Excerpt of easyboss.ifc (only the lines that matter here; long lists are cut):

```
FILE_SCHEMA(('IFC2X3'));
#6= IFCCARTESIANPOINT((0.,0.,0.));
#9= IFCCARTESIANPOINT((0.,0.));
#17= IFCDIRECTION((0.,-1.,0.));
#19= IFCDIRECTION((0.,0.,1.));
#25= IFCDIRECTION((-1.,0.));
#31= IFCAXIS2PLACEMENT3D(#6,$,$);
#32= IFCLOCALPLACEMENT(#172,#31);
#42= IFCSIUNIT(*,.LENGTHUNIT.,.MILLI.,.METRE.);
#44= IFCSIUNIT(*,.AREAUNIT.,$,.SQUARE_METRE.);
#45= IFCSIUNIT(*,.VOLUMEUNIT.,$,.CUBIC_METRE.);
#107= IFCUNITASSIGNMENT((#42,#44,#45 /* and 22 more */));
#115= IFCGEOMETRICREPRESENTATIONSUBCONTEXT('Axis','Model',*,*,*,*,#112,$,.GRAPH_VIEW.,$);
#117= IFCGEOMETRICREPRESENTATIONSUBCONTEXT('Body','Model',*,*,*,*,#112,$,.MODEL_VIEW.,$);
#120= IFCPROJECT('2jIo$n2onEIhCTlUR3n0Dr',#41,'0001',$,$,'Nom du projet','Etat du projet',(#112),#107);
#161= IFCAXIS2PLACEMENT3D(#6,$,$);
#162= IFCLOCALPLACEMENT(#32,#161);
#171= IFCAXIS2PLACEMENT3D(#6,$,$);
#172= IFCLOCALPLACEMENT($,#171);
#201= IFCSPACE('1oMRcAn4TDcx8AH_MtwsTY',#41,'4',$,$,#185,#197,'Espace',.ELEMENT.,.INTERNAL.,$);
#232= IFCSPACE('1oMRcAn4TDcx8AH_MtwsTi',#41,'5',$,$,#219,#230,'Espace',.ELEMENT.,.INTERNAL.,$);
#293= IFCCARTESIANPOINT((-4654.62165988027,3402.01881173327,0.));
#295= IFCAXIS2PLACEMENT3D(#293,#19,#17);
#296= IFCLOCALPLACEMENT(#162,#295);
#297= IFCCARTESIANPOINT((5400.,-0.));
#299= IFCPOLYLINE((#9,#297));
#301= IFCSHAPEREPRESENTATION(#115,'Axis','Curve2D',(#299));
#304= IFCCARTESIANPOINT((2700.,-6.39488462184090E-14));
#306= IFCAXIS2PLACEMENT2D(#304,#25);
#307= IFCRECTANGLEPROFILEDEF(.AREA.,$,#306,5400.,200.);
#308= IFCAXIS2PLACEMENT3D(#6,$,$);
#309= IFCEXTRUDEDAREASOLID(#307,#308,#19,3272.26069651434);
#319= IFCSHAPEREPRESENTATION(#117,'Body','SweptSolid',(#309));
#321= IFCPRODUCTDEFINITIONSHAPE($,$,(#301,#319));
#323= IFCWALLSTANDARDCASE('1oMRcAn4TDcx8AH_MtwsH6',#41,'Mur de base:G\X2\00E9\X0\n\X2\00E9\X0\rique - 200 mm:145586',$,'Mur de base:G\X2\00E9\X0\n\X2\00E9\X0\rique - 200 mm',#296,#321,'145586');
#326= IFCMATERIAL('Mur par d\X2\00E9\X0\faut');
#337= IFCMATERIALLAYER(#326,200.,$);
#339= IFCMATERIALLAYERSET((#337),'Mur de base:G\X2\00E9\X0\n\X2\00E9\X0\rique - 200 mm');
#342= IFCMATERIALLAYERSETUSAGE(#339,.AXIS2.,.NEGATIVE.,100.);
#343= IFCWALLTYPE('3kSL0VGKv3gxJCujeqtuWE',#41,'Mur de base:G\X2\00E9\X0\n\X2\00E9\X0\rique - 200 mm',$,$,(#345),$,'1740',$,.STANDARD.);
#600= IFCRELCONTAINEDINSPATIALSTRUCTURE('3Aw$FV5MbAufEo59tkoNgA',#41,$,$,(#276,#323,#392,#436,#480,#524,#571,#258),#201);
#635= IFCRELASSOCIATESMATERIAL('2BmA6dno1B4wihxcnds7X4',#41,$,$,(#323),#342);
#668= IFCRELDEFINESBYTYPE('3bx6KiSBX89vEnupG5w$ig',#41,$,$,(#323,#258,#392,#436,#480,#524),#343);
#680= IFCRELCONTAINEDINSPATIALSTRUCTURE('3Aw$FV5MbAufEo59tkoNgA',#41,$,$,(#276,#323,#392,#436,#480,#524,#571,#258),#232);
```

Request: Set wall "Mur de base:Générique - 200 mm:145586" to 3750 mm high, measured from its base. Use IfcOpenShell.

```python
import ifcopenshell
import ifcopenshell.geom
import ifcopenshell.util.representation
import ifcopenshell.util.shape

model = ifcopenshell.open("easyboss.ifc")
settings = ifcopenshell.geom.settings()


def volume(element):
    """Net volume in cubic metres, openings subtracted."""
    shape = ifcopenshell.geom.create_shape(settings, element)
    return ifcopenshell.util.shape.get_volume(shape.geometry)


wall = model.by_guid("1oMRcAn4TDcx8AH_MtwsH6")
before = volume(wall)

body = ifcopenshell.util.representation.get_representation(wall, "Model", "Body")
solid = body.Items[0]
old_height = solid.Depth
solid.Depth = 3750.0
after = volume(wall)

print(f"height {old_height:g} -> {solid.Depth:g}, volume {before:.3f} -> {after:.3f} m3")

model.write("easyboss-out.ifc")
```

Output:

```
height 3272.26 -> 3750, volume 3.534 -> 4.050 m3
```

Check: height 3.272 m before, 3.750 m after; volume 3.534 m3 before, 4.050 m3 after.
